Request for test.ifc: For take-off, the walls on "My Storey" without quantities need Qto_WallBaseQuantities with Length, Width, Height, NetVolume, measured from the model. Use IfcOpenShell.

First a look at what the model holds.

```python
import ifcopenshell
import ifcopenshell.util.element
import ifcopenshell.util.unit

model = ifcopenshell.open("test.ifc")
print(model.schema)
for unit_type in ("LENGTHUNIT", "AREAUNIT", "VOLUMEUNIT"):
    print(unit_type, ifcopenshell.util.unit.calculate_unit_scale(model, unit_type))
storey = next(s for s in model.by_type("IfcBuildingStorey") if s.Name == "My Storey")
walls = [e for e in ifcopenshell.util.element.get_decomposition(storey) if e.is_a("IfcWall")]
for e in sorted(walls, key=lambda e: e.id()):
    print(e.id(), e.is_a(), e.Name, list(ifcopenshell.util.element.get_psets(e, qtos_only=True)), sep=" | ")
```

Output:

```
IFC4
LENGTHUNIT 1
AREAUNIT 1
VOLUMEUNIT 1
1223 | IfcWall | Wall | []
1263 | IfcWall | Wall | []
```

```python
import ifcopenshell
import ifcopenshell.api.pset
import ifcopenshell.geom
import ifcopenshell.util.element
import ifcopenshell.util.shape
import ifcopenshell.util.unit

model = ifcopenshell.open("test.ifc")
unit_scale = ifcopenshell.util.unit.calculate_unit_scale(model)
volume_scale = ifcopenshell.util.unit.calculate_unit_scale(model, "VOLUMEUNIT")
settings = ifcopenshell.geom.settings()

storey = next(s for s in model.by_type("IfcBuildingStorey") if s.Name == "My Storey")
walls = [e for e in ifcopenshell.util.element.get_decomposition(storey) if e.is_a("IfcWall")]

for e in sorted(walls, key=lambda e: e.id()):
    if ifcopenshell.util.element.get_psets(e, qtos_only=True, should_inherit=False):
        continue
    # Geometry comes back in metres, in the element's own axes.
    shape = ifcopenshell.geom.create_shape(settings, e)
    values = {
        "Length": ifcopenshell.util.shape.get_x(shape.geometry) / unit_scale,
        "Width": ifcopenshell.util.shape.get_y(shape.geometry) / unit_scale,
        "Height": ifcopenshell.util.shape.get_z(shape.geometry) / unit_scale,
        "NetVolume": ifcopenshell.util.shape.get_volume(shape.geometry) / volume_scale,
    }
    qto = ifcopenshell.api.pset.add_qto(model, product=e, name="Qto_WallBaseQuantities")
    ifcopenshell.api.pset.edit_qto(model, qto=qto, properties=values)
    print(e.id(), {k: round(v, 3) for k, v in values.items()})

model.write("test_updated.ifc")
```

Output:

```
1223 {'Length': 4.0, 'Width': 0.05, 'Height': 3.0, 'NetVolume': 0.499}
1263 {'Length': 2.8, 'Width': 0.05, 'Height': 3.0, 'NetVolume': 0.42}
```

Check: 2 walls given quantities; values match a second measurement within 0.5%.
